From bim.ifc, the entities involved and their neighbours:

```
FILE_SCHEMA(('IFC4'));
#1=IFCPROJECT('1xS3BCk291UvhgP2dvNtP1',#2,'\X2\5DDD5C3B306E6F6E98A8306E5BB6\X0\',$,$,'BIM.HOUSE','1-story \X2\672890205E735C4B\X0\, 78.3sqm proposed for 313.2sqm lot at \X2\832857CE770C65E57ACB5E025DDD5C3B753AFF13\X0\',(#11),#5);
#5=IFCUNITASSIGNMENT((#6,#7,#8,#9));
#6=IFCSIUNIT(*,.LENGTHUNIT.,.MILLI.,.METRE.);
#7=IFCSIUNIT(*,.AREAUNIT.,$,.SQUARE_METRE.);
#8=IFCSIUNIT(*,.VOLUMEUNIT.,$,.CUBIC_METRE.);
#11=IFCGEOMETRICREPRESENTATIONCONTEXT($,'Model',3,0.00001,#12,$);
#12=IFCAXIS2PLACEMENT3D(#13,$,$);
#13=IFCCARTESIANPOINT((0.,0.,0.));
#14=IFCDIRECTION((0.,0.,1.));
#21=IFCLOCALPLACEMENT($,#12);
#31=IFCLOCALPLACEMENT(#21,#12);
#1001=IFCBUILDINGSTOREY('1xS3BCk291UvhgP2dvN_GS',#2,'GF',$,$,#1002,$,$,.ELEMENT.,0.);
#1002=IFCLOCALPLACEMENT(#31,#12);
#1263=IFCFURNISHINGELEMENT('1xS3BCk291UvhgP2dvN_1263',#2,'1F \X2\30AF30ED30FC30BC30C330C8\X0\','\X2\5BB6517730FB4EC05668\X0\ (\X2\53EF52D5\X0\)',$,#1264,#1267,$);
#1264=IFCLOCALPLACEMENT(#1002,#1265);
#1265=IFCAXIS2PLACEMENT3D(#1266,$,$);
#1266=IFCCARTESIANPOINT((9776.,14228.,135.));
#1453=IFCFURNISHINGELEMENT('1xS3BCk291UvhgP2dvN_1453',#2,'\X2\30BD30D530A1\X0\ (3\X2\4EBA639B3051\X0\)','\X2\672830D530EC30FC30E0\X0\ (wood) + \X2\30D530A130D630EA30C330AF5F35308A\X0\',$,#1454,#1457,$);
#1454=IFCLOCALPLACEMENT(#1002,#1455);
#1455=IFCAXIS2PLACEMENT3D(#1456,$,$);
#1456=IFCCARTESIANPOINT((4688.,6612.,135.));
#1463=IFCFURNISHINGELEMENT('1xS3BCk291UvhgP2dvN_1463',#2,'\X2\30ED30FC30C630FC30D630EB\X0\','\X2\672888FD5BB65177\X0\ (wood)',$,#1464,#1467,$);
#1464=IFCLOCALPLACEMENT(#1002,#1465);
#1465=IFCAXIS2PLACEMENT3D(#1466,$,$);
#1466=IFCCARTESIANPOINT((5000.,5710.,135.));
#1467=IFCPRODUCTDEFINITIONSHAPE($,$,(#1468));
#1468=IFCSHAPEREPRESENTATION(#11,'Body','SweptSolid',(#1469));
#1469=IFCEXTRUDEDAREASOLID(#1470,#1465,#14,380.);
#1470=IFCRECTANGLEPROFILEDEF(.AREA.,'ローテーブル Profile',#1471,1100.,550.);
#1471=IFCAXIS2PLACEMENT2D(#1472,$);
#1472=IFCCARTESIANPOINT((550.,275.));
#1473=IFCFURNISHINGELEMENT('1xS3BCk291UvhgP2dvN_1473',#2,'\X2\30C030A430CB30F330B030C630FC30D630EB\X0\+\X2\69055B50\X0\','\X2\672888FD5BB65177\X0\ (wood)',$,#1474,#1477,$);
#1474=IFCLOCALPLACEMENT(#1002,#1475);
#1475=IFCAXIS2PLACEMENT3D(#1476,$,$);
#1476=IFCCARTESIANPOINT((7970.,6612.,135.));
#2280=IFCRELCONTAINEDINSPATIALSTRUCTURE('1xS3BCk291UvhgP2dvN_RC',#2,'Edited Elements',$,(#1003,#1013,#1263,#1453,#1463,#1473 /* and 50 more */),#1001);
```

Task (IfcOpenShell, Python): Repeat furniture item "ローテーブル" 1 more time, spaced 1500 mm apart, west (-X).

```python
import numpy as np
import ifcopenshell
import ifcopenshell.api.geometry
import ifcopenshell.api.root
import ifcopenshell.util.element
import ifcopenshell.util.placement
import ifcopenshell.util.unit

model = ifcopenshell.open("bim.ifc")
unit_scale = ifcopenshell.util.unit.calculate_unit_scale(model)


def reuse_history(source, copy):
    """copy_class also copies each property set's owner history, people and application; keep the originals."""
    for rel in copy.IsDefinedBy:
        if rel.is_a("IfcRelDefinesByProperties") and (history := rel.RelatingPropertyDefinition.OwnerHistory):
            rel.RelatingPropertyDefinition.OwnerHistory = source.OwnerHistory
            ifcopenshell.util.element.remove_deep2(model, history)


source = model.by_guid("1xS3BCk291UvhgP2dvN_1463")
base = ifcopenshell.util.placement.get_local_placement(source.ObjectPlacement)
step = np.array([-1.0, 0.0, 0.0]) * 1.5 / unit_scale

for i in range(1, 2):
    copy = ifcopenshell.api.root.copy_class(model, product=source)
    copy.Representation = ifcopenshell.util.element.copy_deep(
        model, source.Representation, exclude=["IfcGeometricRepresentationContext", "IfcRepresentationMap"]
    )
    reuse_history(source, copy)
    matrix = base.copy()
    matrix[:3, 3] += i * step
    print("added at", matrix[:3, 3].round(3) + 0.0)
    ifcopenshell.api.geometry.edit_object_placement(model, product=copy, matrix=matrix, is_si=False)

model.write("bim-out.ifc")
```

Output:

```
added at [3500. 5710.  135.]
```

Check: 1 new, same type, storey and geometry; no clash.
